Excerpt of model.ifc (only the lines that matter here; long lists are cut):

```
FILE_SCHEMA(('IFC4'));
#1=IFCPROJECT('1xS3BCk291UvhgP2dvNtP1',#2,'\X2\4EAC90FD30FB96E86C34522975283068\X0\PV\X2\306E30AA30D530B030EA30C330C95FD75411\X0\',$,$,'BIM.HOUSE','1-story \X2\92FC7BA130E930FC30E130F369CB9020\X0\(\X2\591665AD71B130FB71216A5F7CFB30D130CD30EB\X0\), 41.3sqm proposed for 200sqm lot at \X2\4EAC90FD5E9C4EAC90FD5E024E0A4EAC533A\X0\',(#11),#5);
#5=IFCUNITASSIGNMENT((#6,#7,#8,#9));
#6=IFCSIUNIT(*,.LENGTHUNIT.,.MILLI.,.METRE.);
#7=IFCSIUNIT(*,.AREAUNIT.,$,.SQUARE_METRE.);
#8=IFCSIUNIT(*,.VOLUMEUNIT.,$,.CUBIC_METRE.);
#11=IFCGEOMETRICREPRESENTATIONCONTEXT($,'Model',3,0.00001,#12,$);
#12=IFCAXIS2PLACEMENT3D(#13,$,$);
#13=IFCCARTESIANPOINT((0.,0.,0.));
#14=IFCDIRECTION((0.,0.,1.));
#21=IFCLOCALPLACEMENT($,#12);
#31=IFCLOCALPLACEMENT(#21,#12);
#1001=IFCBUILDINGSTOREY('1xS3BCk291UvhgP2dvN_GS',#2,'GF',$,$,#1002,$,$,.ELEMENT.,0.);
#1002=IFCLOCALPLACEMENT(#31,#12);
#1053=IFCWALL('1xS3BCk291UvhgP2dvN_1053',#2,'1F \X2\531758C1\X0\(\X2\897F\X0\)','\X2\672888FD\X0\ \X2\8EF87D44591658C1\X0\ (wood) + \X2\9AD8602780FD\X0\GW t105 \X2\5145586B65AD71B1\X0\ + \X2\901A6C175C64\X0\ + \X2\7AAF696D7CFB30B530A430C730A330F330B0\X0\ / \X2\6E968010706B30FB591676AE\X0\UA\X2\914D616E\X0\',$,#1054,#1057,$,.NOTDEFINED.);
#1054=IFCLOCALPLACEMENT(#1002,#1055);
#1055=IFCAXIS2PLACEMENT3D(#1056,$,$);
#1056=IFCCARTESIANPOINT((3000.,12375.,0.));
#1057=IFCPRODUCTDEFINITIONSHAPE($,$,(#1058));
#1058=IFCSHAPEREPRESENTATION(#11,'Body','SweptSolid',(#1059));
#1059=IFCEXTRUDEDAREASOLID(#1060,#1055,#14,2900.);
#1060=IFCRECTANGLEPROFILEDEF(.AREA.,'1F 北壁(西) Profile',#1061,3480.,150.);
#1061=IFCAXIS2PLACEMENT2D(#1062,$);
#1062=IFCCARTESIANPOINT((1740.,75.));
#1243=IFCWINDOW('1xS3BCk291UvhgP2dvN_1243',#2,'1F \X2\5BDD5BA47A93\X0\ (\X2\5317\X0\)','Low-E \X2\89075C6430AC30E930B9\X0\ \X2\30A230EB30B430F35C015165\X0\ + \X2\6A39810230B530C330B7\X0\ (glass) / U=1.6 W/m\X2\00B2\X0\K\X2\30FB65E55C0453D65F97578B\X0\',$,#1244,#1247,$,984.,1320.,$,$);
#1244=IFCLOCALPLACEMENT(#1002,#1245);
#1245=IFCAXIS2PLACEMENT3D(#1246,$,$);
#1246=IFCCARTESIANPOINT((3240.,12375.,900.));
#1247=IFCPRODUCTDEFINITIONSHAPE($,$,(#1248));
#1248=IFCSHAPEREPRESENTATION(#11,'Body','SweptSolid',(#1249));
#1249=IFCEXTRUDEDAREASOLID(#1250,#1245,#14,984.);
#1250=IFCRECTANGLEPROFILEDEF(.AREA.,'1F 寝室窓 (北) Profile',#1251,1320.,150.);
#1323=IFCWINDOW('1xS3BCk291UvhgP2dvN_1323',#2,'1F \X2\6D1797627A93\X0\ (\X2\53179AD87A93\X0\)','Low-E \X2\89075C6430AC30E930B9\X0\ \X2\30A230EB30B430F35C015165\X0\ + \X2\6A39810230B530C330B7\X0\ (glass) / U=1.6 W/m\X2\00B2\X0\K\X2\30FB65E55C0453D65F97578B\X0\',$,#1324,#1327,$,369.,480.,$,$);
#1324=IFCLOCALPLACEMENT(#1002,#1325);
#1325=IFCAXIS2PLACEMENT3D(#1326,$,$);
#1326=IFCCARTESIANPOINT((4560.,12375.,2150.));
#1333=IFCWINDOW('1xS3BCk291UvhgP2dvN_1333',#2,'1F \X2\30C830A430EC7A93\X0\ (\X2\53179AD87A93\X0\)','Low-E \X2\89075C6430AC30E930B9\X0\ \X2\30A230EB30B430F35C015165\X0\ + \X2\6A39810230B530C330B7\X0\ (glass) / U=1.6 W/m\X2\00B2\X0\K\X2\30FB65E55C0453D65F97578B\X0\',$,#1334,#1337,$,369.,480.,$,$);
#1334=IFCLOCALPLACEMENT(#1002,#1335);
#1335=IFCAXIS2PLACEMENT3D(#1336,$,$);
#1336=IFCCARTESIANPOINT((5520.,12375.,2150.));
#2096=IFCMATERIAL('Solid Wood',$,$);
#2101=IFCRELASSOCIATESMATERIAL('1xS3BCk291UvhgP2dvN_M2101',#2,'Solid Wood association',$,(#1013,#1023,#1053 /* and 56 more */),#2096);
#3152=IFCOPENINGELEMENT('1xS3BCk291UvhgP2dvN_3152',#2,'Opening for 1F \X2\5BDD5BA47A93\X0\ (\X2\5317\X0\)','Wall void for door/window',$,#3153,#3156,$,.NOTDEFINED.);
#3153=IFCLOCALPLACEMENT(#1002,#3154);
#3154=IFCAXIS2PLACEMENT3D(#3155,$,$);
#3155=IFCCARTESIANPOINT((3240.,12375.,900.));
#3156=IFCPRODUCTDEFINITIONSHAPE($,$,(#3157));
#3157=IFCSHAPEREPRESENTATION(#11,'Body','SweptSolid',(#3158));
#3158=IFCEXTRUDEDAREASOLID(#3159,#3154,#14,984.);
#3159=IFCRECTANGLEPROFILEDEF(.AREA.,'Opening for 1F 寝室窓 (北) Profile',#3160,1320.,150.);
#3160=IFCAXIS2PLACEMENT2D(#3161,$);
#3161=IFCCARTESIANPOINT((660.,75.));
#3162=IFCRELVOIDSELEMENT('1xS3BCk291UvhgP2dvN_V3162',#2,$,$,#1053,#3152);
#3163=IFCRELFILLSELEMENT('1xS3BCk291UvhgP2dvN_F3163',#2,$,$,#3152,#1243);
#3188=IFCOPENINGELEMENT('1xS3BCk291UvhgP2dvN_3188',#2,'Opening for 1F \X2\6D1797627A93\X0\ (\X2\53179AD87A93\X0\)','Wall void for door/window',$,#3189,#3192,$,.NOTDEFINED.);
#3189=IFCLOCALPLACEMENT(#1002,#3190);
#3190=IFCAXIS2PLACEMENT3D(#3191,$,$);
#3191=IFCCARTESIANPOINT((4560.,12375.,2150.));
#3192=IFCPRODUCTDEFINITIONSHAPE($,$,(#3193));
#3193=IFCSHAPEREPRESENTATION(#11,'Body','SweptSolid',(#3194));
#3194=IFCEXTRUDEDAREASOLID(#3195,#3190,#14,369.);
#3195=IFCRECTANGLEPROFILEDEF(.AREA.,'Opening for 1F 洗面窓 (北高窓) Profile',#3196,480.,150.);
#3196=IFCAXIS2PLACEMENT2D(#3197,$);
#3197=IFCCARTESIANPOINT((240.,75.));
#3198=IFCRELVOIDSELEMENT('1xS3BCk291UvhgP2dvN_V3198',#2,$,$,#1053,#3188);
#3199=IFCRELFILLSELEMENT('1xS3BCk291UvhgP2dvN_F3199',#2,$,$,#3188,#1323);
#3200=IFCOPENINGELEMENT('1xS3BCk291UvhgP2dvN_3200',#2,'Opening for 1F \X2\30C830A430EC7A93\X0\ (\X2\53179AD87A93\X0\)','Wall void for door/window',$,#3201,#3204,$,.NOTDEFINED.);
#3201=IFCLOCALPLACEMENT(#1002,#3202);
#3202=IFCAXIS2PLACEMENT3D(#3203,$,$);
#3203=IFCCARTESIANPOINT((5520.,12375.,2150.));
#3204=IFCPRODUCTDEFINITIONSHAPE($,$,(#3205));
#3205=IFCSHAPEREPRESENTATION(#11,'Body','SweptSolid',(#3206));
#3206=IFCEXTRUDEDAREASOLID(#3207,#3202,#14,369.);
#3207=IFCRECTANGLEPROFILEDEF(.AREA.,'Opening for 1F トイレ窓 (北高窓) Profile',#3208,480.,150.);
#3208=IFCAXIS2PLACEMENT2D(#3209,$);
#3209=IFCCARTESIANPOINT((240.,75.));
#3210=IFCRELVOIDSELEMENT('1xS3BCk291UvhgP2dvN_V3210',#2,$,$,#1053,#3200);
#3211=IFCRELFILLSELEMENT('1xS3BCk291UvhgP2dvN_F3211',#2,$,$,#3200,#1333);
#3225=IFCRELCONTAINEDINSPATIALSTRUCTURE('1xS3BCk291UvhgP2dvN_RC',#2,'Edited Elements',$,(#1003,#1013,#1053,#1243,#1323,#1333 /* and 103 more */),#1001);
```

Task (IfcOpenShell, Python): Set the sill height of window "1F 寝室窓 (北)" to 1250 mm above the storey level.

```python
import numpy as np
import ifcopenshell
import ifcopenshell.api.geometry
import ifcopenshell.geom
import ifcopenshell.util.element
import ifcopenshell.util.placement
import ifcopenshell.util.shape
import ifcopenshell.util.unit

model = ifcopenshell.open("model.ifc")
unit_scale = ifcopenshell.util.unit.calculate_unit_scale(model)

window = model.by_id(1243)
opening = window.FillsVoids[0].RelatingOpeningElement
storey = ifcopenshell.util.element.get_container(window, ifc_class="IfcBuildingStorey")
level = ifcopenshell.util.placement.get_local_placement(storey.ObjectPlacement)[2, 3]

# The opening's origin need not be at the sill, so measure its lowest point.
shape = ifcopenshell.geom.create_shape(ifcopenshell.geom.settings(), opening)
bottom = ifcopenshell.util.shape.get_shape_bottom_elevation(shape, shape.geometry) / unit_scale
dz = level + 1.25 / unit_scale - bottom

shift = np.array([0.0, 0.0, dz])
# The window is not placed relative to its opening, so move both.
for product in (opening, window):
    matrix = ifcopenshell.util.placement.get_local_placement(product.ObjectPlacement)
    matrix[:3, 3] += shift
    ifcopenshell.api.geometry.edit_object_placement(model, product=product, matrix=matrix, is_si=False)

print(f"moved by {dz * unit_scale:+.3f} m")

model.write("model_rev.ifc")
```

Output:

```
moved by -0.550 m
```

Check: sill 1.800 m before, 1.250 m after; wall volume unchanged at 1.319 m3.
